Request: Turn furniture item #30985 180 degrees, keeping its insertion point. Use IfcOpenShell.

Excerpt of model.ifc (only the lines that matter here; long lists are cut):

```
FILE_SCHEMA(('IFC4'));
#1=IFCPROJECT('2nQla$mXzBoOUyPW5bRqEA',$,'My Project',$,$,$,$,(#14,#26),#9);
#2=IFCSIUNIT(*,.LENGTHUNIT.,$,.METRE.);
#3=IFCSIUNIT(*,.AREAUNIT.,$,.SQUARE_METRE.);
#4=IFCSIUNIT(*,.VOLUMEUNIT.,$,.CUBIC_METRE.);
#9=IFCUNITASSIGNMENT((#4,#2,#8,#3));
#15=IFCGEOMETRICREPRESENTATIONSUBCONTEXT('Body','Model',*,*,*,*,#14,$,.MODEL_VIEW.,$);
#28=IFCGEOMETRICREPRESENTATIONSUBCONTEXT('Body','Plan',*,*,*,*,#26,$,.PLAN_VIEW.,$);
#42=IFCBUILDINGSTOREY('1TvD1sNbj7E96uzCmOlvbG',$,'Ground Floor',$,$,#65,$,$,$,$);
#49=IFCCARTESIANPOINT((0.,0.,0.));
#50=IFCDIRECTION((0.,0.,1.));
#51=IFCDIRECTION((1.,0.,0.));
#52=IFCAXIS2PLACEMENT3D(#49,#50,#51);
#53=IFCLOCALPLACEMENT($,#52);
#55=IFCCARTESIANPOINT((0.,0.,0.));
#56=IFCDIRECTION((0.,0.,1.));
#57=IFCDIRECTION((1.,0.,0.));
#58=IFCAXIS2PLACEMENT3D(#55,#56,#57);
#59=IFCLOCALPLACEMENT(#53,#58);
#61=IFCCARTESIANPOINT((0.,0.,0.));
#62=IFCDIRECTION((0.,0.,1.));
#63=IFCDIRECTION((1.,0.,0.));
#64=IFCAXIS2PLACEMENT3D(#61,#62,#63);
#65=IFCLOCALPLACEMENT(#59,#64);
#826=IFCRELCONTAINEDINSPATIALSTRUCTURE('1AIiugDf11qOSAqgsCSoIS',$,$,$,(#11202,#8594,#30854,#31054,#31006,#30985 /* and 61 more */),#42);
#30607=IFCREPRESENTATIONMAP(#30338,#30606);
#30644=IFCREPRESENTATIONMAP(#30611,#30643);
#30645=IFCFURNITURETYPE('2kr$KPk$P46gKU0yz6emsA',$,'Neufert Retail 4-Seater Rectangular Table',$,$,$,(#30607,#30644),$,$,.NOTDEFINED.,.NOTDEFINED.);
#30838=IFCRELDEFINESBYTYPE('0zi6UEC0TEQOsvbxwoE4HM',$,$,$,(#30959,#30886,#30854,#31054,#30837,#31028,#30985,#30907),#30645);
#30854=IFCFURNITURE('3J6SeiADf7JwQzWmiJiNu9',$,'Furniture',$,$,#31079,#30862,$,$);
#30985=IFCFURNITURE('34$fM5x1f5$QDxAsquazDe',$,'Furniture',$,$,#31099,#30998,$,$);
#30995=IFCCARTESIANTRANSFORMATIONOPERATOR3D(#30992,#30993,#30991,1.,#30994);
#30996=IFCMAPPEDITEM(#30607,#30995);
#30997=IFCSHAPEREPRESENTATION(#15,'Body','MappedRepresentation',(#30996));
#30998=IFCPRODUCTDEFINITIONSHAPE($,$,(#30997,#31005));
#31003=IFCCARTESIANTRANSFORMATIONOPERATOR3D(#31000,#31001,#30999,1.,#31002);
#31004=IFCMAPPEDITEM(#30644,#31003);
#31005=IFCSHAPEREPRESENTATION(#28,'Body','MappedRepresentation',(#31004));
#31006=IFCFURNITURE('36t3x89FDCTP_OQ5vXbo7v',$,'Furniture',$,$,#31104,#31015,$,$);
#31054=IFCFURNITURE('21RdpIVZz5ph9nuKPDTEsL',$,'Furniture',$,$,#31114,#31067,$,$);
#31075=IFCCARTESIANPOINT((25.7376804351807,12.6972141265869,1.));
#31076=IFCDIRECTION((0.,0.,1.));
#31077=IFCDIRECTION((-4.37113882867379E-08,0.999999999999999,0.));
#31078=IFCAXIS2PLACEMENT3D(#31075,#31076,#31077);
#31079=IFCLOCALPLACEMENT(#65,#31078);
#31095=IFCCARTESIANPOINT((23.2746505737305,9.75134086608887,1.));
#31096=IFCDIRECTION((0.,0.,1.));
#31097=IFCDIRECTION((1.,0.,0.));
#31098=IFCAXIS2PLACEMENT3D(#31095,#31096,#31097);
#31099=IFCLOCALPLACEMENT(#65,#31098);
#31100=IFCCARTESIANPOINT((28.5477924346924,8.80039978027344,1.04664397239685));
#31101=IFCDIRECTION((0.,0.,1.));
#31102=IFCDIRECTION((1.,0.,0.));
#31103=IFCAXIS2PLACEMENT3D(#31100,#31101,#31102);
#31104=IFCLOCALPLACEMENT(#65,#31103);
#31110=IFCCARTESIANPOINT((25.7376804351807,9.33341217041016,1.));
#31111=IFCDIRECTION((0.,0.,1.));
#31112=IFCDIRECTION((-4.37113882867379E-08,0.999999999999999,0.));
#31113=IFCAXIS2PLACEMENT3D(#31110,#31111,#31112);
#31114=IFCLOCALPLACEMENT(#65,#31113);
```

```python
import ifcopenshell
import ifcopenshell.api.geometry
import ifcopenshell.util.placement

model = ifcopenshell.open("model.ifc")

item = model.by_guid("34$fM5x1f5$QDxAsquazDe")
matrix = ifcopenshell.util.placement.get_local_placement(item.ObjectPlacement)
matrix = matrix @ ifcopenshell.util.placement.rotation(180, "Z")
ifcopenshell.api.geometry.edit_object_placement(model, product=item, matrix=matrix, is_si=False)

print(ifcopenshell.util.placement.get_local_placement(item.ObjectPlacement).round(3) + 0.0)

model.write("model-out.ifc")
```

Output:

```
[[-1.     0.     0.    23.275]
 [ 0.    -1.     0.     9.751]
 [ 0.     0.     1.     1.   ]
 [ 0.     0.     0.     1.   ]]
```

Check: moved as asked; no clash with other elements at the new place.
